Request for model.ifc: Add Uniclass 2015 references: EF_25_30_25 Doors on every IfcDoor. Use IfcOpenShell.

First a look at what the model holds.

```python
import ifcopenshell

model = ifcopenshell.open("model.ifc")
print(model.schema)
print("classifications:", [c.Name for c in model.by_type("IfcClassification")])
for ifc_class in ("IfcDoor", "IfcRoof", "IfcStair", "IfcWall", "IfcWindow"):
    print(ifc_class, len(model.by_type(ifc_class)))
```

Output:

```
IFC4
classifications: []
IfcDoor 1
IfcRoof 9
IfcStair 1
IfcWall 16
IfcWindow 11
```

```python
import ifcopenshell
import ifcopenshell.api.classification

model = ifcopenshell.open("model.ifc")

system = ifcopenshell.api.classification.add_classification(model, classification="Uniclass 2015")

codes = {
    "IfcDoor": ("EF_25_30_25", "Doors"),
}
for ifc_class, (code, name) in codes.items():
    products = model.by_type(ifc_class)
    ifcopenshell.api.classification.add_reference(
        model, products=products, classification=system, identification=code, name=name
    )
    print(code, len(products))

model.write("model_rev.ifc")
```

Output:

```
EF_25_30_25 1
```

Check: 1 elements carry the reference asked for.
